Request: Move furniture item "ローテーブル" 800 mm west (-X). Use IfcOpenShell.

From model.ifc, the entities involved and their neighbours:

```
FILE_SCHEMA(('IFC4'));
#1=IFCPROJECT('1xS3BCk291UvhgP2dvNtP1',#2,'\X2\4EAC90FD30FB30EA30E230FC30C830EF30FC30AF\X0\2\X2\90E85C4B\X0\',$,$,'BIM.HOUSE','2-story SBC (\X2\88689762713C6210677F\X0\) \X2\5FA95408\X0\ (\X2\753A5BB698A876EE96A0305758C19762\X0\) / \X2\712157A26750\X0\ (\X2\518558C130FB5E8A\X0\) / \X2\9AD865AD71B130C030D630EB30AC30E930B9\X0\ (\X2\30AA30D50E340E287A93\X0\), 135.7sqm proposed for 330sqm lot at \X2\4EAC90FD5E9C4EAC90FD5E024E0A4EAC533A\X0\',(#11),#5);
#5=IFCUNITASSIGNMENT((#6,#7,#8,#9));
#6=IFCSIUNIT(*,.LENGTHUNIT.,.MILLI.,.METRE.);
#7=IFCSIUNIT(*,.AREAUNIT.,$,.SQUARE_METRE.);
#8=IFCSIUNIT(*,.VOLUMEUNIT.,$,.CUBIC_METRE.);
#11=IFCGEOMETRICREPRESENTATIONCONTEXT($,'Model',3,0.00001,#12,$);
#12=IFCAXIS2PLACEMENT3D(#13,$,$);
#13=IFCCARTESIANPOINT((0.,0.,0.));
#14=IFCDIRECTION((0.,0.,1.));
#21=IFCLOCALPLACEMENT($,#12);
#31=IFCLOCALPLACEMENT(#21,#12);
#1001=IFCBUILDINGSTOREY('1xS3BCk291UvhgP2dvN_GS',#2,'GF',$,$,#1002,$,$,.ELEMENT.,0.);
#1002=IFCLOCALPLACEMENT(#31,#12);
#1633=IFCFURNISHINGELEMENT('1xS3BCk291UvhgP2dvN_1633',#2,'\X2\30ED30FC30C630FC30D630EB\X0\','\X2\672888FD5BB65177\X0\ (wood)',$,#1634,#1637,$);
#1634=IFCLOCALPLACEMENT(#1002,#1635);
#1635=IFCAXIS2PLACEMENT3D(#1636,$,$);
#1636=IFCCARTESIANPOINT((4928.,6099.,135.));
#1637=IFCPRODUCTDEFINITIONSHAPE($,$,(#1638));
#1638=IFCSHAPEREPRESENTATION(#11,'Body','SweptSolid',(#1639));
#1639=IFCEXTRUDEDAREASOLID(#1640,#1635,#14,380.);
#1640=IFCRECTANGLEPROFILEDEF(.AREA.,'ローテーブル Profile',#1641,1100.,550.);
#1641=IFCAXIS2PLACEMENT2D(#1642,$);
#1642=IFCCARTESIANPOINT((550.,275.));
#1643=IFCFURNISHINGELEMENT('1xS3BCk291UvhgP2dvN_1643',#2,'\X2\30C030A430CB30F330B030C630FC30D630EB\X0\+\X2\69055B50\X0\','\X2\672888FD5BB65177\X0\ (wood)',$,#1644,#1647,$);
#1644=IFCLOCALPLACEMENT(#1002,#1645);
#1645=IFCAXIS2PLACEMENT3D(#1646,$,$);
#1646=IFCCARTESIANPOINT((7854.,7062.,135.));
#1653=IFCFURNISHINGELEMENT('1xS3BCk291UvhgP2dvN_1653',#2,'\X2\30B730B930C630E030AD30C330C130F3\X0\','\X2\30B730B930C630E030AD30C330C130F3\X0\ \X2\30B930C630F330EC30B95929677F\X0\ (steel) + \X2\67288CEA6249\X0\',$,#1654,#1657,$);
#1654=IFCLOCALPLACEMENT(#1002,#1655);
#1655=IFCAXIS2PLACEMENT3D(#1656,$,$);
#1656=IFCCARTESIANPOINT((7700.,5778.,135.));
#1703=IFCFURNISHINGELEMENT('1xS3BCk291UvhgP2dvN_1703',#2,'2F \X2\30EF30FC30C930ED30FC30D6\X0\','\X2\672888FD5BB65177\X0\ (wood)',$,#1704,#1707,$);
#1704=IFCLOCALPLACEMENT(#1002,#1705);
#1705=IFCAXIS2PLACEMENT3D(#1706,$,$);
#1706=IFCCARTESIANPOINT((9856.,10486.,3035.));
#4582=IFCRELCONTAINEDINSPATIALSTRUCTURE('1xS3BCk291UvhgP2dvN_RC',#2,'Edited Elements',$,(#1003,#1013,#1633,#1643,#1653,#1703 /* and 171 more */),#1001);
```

```python
import ifcopenshell
import ifcopenshell.api.geometry
import ifcopenshell.util.placement
import ifcopenshell.util.unit

model = ifcopenshell.open("model.ifc")
unit_scale = ifcopenshell.util.unit.calculate_unit_scale(model)

item = model.by_id(1633)
matrix = ifcopenshell.util.placement.get_local_placement(item.ObjectPlacement)
matrix[0, 3] -= 0.8 / unit_scale
ifcopenshell.api.geometry.edit_object_placement(model, product=item, matrix=matrix, is_si=False)

print(ifcopenshell.util.placement.get_local_placement(item.ObjectPlacement).round(3) + 0.0)

model.write("model_v2.ifc")
```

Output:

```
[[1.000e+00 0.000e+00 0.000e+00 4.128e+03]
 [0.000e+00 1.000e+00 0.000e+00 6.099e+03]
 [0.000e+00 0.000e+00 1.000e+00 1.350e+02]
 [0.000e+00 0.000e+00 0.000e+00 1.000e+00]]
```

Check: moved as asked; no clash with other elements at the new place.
